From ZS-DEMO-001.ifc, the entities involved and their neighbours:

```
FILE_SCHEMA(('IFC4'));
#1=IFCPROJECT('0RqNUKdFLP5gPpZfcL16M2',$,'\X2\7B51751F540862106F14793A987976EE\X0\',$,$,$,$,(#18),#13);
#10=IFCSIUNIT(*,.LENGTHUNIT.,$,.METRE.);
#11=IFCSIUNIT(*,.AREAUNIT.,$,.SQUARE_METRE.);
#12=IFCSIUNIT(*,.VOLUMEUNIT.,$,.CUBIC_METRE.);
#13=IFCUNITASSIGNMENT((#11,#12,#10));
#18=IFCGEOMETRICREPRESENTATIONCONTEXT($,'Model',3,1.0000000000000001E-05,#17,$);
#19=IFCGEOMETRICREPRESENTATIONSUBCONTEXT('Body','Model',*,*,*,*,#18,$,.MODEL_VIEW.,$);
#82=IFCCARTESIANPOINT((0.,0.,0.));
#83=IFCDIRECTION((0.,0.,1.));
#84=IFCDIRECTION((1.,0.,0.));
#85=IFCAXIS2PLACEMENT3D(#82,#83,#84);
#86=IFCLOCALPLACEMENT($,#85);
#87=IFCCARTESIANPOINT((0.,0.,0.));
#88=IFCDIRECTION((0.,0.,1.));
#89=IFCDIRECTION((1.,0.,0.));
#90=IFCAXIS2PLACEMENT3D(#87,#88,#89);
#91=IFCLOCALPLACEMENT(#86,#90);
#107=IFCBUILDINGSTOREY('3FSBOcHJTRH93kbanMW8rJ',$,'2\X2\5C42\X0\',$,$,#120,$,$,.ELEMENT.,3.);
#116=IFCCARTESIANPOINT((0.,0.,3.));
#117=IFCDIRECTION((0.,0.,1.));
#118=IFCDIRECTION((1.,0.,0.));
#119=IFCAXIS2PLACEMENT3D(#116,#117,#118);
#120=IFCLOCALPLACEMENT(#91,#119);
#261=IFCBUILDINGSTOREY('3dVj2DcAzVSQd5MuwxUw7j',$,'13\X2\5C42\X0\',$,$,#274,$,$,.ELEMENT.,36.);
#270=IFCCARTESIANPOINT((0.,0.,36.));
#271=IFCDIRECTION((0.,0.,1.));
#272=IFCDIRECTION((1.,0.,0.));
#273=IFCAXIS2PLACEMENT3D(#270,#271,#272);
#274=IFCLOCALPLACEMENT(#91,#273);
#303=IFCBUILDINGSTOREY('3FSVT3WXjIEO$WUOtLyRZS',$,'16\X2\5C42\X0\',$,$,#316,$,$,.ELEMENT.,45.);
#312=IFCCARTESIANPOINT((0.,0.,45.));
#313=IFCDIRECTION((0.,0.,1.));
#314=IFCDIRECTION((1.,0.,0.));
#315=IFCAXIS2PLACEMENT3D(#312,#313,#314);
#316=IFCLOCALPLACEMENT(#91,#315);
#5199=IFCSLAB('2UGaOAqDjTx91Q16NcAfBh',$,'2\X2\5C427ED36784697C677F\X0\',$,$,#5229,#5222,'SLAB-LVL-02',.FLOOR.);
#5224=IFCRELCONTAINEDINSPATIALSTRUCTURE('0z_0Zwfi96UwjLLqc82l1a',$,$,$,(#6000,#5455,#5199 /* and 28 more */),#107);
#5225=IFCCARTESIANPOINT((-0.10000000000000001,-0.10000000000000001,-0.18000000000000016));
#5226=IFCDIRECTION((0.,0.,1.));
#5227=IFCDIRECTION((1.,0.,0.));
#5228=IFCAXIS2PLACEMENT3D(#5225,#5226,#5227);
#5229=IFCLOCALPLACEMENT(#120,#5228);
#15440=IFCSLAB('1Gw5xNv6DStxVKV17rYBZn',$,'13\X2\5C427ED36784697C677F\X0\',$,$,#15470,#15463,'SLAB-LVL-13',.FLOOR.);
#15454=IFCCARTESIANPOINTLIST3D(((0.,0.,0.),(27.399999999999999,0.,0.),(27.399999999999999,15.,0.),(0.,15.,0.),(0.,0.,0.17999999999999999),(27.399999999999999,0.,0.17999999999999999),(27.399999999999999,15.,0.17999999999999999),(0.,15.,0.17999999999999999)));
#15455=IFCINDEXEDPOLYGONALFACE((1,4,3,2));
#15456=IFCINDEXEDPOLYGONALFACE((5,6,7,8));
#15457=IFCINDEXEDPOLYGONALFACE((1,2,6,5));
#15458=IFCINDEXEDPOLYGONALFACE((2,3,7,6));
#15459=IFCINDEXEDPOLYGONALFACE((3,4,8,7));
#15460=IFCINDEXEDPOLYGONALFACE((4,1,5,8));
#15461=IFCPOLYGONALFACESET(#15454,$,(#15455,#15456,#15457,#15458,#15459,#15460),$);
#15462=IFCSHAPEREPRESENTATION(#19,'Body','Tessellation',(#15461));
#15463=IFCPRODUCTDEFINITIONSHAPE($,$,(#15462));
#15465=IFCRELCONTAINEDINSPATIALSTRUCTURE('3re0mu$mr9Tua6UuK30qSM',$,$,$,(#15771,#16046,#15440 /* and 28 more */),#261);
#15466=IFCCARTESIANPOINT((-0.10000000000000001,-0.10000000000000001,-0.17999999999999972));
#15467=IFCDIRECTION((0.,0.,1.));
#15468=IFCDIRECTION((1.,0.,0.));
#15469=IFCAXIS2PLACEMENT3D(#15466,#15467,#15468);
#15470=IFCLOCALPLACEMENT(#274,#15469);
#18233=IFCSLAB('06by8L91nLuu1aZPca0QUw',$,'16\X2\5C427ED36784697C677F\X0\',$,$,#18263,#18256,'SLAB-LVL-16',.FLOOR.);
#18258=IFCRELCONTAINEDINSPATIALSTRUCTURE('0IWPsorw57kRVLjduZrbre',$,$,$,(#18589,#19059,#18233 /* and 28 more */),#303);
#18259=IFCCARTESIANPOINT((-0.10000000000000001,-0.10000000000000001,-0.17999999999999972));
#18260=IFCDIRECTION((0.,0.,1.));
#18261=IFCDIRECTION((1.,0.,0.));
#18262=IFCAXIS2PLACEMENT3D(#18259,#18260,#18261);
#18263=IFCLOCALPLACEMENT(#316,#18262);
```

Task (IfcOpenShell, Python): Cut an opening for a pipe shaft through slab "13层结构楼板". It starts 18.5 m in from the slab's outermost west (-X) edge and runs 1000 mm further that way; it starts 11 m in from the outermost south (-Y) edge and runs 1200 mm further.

```python
import numpy as np
import ifcopenshell
import ifcopenshell.api.feature
import ifcopenshell.api.geometry
import ifcopenshell.api.root
import ifcopenshell.geom
import ifcopenshell.util.placement
import ifcopenshell.util.representation
import ifcopenshell.util.shape
import ifcopenshell.util.unit

model = ifcopenshell.open("ZS-DEMO-001.ifc")
unit_scale = ifcopenshell.util.unit.calculate_unit_scale(model)
settings = ifcopenshell.geom.settings()


def volume(element):
    """Net volume in cubic metres, openings subtracted."""
    shape = ifcopenshell.geom.create_shape(settings, element)
    return ifcopenshell.util.shape.get_volume(shape.geometry)


slab = model.by_guid("1Gw5xNv6DStxVKV17rYBZn")
before = volume(slab)

# Extent in the slab's own axes, in metres. The edges named are its -X and -Y sides.
slab_shape = ifcopenshell.geom.create_shape(settings, slab)
vertices = ifcopenshell.util.shape.get_vertices(slab_shape.geometry)
x_min, y_min, bottom = vertices.min(axis=0)
top = vertices[:, 2].max()

opening = ifcopenshell.api.root.create_entity(model, ifc_class="IfcOpeningElement", name="Pipe shaft opening", predefined_type="OPENING")
context = ifcopenshell.util.representation.get_context(model, "Model", "Body", "MODEL_VIEW")
width, depth = 1, 1.2
outline = [(0.0, 0.0), (width, 0.0), (width, depth), (0.0, depth), (0.0, 0.0)]
# Overshoot both faces by 50 mm so the cut is clean.
shape = ifcopenshell.api.geometry.add_slab_representation(
    model, context=context, depth=top - bottom + 0.1, polyline=outline
)
ifcopenshell.api.geometry.assign_representation(model, product=opening, representation=shape)

matrix = ifcopenshell.util.placement.get_local_placement(slab.ObjectPlacement)
matrix[:, 3] = matrix @ np.append(np.array([x_min + 18.5, y_min + 11, bottom - 0.05]) / unit_scale, 1.0)
ifcopenshell.api.geometry.edit_object_placement(model, product=opening, matrix=matrix, is_si=False)
ifcopenshell.api.feature.add_feature(model, feature=opening, element=slab)

after = volume(slab)

print(f"slab volume {before:.3f} -> {after:.3f} m3")

model.write("ZS-DEMO-001_updated.ifc")
```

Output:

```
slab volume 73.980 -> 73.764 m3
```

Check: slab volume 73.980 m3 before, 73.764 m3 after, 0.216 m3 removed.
